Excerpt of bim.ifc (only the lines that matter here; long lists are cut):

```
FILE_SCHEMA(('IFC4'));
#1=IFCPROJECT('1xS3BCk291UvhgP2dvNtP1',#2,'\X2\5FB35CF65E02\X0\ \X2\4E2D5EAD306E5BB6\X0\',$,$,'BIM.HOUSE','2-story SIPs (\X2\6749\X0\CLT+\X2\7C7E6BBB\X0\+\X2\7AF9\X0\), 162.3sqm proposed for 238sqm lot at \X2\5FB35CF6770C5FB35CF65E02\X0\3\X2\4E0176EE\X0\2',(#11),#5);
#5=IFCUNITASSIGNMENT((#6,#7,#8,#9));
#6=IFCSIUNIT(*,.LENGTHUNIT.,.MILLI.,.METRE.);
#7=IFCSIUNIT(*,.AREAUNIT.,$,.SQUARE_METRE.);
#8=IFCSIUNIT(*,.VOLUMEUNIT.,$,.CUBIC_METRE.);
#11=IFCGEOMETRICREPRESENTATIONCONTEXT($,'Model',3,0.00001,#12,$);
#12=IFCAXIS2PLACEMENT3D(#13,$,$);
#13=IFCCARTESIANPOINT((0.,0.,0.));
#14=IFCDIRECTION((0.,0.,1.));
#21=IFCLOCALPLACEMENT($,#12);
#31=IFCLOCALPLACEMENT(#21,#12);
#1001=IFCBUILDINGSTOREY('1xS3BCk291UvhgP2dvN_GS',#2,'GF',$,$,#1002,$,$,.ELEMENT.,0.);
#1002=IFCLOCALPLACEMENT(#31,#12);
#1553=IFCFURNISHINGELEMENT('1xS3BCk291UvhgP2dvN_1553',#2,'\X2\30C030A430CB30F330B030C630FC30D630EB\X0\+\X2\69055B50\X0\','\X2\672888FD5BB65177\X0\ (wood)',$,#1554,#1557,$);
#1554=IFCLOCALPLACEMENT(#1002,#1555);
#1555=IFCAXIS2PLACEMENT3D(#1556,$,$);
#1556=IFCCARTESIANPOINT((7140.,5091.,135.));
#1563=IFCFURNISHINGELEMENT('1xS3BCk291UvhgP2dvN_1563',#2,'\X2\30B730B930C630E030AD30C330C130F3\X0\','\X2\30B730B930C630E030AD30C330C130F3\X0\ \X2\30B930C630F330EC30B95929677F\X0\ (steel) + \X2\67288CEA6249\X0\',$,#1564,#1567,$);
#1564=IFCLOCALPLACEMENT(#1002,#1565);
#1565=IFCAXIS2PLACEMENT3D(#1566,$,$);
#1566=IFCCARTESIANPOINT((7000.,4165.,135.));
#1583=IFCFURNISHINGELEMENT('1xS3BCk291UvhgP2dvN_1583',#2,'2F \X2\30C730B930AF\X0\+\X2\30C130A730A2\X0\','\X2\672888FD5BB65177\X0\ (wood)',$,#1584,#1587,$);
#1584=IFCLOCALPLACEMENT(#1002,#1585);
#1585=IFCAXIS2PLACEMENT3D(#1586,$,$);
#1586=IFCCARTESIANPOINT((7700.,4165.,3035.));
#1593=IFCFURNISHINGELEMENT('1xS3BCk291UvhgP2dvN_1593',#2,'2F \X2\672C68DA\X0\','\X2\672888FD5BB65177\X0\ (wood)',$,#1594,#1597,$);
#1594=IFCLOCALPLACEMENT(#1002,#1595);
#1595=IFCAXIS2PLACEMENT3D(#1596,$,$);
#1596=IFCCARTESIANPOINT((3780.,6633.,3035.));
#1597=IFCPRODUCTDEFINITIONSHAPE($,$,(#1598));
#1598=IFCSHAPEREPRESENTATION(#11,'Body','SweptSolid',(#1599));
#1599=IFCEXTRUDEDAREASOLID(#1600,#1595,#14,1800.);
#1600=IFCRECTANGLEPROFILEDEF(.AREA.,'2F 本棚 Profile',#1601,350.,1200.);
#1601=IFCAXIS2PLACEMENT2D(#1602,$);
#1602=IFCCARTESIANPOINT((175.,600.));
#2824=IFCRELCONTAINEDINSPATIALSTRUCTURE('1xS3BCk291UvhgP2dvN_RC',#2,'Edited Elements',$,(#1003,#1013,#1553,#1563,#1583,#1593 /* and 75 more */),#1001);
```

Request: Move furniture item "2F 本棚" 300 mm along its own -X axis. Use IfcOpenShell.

```python
import ifcopenshell
import ifcopenshell.api.geometry
import ifcopenshell.util.placement

model = ifcopenshell.open("bim.ifc")

item = model.by_guid("1xS3BCk291UvhgP2dvN_1593")
matrix = ifcopenshell.util.placement.get_local_placement(item.ObjectPlacement)
matrix[:3, 3] -= matrix[:3, 0] * 300.0
ifcopenshell.api.geometry.edit_object_placement(model, product=item, matrix=matrix, is_si=False)

print(ifcopenshell.util.placement.get_local_placement(item.ObjectPlacement).round(3) + 0.0)

model.write("bim-out.ifc")
```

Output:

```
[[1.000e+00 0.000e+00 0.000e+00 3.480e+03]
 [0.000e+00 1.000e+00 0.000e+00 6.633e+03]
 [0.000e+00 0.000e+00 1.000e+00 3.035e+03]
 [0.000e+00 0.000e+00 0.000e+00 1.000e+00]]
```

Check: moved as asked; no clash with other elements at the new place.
